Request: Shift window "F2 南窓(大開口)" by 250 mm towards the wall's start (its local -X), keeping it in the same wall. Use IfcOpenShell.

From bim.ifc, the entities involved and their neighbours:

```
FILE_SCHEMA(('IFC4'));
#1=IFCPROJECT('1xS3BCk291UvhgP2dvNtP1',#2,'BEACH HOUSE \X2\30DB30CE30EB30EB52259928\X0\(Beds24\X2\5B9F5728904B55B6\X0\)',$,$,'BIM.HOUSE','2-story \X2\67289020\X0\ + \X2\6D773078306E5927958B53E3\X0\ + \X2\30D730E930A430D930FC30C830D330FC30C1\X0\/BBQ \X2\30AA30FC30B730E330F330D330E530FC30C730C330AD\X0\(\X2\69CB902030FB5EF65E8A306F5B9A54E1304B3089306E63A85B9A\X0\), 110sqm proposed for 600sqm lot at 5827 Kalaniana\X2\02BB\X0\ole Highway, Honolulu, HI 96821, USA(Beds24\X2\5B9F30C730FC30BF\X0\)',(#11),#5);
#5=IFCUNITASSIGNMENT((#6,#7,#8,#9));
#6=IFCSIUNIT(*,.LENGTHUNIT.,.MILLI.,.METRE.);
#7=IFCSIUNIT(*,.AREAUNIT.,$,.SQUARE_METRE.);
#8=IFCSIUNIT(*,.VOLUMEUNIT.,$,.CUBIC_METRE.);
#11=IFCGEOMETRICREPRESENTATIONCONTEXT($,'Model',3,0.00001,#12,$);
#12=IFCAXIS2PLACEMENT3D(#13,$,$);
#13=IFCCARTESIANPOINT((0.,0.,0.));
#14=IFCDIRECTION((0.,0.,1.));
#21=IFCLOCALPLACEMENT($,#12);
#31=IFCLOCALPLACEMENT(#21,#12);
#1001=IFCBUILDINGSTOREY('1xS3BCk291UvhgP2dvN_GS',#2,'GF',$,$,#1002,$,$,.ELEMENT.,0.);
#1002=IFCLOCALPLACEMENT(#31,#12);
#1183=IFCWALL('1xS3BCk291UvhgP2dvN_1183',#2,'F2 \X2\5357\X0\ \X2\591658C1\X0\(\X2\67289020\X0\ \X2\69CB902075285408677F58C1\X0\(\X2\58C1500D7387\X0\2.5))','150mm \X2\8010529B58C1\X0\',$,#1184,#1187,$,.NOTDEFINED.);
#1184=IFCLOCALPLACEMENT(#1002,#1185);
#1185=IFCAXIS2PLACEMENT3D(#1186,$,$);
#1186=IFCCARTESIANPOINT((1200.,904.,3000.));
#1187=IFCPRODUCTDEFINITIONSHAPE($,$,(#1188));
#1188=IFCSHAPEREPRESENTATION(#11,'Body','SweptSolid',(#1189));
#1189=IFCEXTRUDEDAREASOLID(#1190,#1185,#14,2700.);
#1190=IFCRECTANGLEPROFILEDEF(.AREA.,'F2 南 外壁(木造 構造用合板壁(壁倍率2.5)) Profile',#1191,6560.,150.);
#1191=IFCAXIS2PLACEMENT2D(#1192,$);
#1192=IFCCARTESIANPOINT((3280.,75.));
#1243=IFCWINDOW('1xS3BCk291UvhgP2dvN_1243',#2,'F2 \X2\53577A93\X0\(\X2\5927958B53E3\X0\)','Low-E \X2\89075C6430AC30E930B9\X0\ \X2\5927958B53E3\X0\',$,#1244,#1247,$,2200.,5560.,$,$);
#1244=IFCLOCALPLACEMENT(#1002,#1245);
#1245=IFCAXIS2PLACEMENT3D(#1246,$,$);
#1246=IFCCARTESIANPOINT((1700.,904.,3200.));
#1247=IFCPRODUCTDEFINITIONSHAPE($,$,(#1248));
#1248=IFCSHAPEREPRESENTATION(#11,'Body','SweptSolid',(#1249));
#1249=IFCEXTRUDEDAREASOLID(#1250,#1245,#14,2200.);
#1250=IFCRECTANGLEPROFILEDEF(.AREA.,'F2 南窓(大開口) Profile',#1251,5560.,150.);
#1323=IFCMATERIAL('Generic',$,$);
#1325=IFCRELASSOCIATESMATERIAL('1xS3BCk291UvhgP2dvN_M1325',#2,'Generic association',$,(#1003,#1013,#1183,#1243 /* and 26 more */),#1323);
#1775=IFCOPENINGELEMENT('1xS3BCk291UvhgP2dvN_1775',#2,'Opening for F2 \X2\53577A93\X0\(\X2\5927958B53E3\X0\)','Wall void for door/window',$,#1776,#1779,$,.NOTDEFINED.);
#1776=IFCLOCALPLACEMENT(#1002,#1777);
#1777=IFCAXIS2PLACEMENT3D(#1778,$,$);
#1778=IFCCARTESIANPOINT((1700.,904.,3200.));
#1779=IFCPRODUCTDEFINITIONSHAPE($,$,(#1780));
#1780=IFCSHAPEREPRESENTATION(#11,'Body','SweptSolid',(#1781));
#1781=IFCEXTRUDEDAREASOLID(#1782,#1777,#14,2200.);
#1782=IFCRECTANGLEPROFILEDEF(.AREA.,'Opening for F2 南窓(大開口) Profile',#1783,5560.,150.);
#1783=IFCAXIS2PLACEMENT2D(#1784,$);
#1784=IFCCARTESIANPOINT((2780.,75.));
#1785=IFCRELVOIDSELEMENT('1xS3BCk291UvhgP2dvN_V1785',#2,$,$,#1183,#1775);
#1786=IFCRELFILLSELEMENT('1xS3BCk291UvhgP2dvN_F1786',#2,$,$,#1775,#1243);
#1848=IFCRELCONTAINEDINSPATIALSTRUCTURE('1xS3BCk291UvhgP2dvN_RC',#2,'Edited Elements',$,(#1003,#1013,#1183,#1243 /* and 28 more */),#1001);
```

```python
import ifcopenshell
import ifcopenshell.api.geometry
import ifcopenshell.util.placement
import ifcopenshell.util.unit

model = ifcopenshell.open("bim.ifc")
unit_scale = ifcopenshell.util.unit.calculate_unit_scale(model)

window = model.by_id(1243)
opening = window.FillsVoids[0].RelatingOpeningElement
wall = opening.VoidsElements[0].RelatingBuildingElement

wall_matrix = ifcopenshell.util.placement.get_local_placement(wall.ObjectPlacement)
shift = wall_matrix[:3, 0] * -0.25 / unit_scale
before = ifcopenshell.util.placement.get_local_placement(window.ObjectPlacement)[:3, 3].copy()

# The window is not placed relative to its opening, so move both.
for product in (opening, window):
    matrix = ifcopenshell.util.placement.get_local_placement(product.ObjectPlacement)
    matrix[:3, 3] += shift
    ifcopenshell.api.geometry.edit_object_placement(model, product=product, matrix=matrix, is_si=False)

after = ifcopenshell.util.placement.get_local_placement(window.ObjectPlacement)[:3, 3]
print("window moved by", (after - before).round(3) + 0.0)

model.write("bim_edited.ifc")
```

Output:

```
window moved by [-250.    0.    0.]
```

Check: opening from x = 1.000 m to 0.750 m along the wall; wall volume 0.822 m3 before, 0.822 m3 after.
